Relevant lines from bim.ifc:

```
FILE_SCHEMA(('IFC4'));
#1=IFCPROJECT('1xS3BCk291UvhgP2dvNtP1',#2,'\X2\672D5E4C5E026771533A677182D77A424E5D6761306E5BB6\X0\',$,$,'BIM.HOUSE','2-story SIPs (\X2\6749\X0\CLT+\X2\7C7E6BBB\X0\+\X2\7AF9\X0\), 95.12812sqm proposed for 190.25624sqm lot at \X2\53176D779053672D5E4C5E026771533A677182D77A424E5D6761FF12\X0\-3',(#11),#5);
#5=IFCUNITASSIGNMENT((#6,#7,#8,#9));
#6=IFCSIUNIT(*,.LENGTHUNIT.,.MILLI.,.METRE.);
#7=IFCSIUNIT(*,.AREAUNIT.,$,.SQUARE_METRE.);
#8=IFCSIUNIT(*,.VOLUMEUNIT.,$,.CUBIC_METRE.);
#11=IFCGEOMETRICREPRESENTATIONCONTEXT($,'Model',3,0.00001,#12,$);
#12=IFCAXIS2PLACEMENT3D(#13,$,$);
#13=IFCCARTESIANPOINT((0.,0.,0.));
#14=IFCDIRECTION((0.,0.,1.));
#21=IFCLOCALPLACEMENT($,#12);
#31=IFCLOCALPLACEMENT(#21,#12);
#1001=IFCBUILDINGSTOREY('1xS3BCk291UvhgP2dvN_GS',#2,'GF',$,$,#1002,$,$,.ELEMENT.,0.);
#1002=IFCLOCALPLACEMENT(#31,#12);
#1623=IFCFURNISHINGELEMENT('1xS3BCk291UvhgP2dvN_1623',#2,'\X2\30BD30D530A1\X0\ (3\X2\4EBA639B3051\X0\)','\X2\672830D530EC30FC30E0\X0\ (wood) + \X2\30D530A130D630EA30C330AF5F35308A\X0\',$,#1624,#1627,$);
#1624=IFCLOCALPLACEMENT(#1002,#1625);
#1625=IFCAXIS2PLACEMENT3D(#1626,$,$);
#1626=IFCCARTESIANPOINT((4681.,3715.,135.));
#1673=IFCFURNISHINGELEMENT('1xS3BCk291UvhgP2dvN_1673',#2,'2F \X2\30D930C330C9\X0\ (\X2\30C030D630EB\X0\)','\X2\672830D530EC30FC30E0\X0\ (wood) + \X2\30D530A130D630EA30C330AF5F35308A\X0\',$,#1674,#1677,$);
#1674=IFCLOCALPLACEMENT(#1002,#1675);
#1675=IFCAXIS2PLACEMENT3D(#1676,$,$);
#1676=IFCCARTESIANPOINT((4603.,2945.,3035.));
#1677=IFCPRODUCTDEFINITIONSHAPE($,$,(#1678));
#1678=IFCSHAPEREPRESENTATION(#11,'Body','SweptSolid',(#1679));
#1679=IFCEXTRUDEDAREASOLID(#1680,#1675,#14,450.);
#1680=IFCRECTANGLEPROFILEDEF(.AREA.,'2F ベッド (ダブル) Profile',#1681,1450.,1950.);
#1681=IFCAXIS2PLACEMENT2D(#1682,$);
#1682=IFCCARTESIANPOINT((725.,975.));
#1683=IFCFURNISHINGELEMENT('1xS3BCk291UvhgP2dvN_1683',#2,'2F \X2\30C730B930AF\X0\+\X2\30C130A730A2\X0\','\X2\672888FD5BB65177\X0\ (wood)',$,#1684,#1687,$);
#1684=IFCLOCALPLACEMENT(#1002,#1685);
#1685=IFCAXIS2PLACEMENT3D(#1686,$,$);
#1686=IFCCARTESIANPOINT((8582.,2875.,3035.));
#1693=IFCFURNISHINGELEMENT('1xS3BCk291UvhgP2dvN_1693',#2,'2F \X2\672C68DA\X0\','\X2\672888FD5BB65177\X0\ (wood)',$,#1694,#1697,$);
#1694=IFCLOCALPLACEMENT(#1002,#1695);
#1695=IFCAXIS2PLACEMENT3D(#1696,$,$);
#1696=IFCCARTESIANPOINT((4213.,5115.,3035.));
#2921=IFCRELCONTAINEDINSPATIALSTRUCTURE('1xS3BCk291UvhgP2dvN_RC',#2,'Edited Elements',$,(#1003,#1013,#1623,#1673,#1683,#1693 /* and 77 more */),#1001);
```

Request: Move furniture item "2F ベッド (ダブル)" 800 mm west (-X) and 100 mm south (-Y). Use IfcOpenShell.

```python
import ifcopenshell
import ifcopenshell.api.geometry
import ifcopenshell.util.placement

model = ifcopenshell.open("bim.ifc")

item = model.by_id(1673)
matrix = ifcopenshell.util.placement.get_local_placement(item.ObjectPlacement)
matrix[0, 3] -= 800.0
matrix[1, 3] -= 100.0
ifcopenshell.api.geometry.edit_object_placement(model, product=item, matrix=matrix, is_si=False)

print(ifcopenshell.util.placement.get_local_placement(item.ObjectPlacement).round(3) + 0.0)

model.write("bim-out.ifc")
```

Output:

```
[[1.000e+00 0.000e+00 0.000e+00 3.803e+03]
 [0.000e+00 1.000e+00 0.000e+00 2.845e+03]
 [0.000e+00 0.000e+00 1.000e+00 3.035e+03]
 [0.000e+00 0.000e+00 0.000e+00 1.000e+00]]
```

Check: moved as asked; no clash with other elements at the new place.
